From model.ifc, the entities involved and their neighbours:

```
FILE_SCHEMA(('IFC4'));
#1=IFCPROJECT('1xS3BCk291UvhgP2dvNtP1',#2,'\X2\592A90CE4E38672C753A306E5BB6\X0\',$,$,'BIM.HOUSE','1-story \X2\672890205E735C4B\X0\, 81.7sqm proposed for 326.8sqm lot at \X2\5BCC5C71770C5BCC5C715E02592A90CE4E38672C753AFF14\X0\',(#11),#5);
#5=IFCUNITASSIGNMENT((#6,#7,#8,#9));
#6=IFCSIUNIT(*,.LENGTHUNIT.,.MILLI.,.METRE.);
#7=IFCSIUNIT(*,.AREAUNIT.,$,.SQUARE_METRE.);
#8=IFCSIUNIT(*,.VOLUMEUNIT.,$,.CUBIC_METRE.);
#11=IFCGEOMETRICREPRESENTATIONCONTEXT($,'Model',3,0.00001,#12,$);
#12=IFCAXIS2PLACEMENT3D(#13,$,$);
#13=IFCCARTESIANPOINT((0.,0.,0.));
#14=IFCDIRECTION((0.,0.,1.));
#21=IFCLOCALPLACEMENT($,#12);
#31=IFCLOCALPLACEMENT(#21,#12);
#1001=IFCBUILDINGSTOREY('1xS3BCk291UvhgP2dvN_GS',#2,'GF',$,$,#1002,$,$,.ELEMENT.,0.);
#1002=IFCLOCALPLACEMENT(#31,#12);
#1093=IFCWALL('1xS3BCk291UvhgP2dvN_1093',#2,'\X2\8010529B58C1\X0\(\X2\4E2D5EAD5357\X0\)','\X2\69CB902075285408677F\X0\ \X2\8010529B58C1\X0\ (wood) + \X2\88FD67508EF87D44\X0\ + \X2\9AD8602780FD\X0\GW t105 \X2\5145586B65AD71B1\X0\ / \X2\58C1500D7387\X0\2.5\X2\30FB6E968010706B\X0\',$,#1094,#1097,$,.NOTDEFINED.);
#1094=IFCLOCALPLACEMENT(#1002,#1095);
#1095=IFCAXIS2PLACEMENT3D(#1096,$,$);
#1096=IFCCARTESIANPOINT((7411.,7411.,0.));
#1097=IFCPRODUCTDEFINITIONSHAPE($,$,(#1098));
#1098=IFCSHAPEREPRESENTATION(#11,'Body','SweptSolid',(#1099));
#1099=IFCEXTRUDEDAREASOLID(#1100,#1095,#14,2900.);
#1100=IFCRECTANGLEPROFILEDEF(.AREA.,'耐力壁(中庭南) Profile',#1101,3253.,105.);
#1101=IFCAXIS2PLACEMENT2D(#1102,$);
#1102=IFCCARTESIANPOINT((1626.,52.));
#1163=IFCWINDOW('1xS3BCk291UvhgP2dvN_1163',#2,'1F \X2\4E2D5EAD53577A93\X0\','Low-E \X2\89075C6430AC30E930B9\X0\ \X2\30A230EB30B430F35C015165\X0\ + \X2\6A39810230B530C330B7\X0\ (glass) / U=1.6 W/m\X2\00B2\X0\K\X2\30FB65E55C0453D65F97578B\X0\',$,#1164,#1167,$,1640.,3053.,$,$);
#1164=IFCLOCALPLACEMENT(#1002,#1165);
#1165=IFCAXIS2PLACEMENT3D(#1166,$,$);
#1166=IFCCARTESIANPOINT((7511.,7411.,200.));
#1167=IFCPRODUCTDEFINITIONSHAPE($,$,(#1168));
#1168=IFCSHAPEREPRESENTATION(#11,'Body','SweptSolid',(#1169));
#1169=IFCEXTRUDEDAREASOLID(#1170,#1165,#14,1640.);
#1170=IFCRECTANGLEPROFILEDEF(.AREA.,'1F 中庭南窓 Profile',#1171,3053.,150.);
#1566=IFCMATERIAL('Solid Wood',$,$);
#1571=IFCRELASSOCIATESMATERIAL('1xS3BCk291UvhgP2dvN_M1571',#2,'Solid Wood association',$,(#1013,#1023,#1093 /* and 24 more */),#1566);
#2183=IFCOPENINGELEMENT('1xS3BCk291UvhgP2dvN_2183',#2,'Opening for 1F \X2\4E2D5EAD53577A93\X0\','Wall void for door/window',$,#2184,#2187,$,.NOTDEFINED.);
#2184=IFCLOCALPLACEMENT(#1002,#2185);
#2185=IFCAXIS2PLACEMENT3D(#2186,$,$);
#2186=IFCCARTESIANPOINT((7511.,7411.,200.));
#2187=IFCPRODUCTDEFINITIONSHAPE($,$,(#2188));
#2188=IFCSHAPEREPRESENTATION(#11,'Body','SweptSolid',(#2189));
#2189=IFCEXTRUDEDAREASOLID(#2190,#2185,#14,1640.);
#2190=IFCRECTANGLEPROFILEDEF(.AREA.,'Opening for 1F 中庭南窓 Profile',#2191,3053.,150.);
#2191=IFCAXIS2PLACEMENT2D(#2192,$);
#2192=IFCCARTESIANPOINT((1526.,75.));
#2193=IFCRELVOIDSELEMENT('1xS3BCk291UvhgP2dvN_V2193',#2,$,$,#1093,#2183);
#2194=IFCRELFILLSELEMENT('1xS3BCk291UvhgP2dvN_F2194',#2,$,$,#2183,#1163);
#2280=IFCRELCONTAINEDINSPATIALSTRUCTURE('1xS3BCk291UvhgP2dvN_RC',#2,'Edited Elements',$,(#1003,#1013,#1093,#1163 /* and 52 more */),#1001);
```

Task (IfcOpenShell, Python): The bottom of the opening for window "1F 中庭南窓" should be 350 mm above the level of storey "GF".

```python
import numpy as np
import ifcopenshell
import ifcopenshell.api.geometry
import ifcopenshell.geom
import ifcopenshell.util.element
import ifcopenshell.util.placement
import ifcopenshell.util.shape
import ifcopenshell.util.unit

model = ifcopenshell.open("model.ifc")
unit_scale = ifcopenshell.util.unit.calculate_unit_scale(model)

window = model.by_guid("1xS3BCk291UvhgP2dvN_1163")
opening = window.FillsVoids[0].RelatingOpeningElement
storey = ifcopenshell.util.element.get_container(window, ifc_class="IfcBuildingStorey")
level = ifcopenshell.util.placement.get_local_placement(storey.ObjectPlacement)[2, 3]

# The opening's origin need not be at the sill, so measure its lowest point.
shape = ifcopenshell.geom.create_shape(ifcopenshell.geom.settings(), opening)
bottom = ifcopenshell.util.shape.get_shape_bottom_elevation(shape, shape.geometry) / unit_scale
dz = level + 350.0 - bottom

shift = np.array([0.0, 0.0, dz])
# The window is not placed relative to its opening, so move both.
for product in (opening, window):
    matrix = ifcopenshell.util.placement.get_local_placement(product.ObjectPlacement)
    matrix[:3, 3] += shift
    ifcopenshell.api.geometry.edit_object_placement(model, product=product, matrix=matrix, is_si=False)

print(f"moved by {dz * unit_scale:+.3f} m")

model.write("model_edited.ifc")
```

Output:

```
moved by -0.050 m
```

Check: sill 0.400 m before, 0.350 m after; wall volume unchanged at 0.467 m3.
